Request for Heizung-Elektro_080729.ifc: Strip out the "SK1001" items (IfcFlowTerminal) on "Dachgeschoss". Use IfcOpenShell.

First a look at what the model holds.

```python
import ifcopenshell
import ifcopenshell.util.element

model = ifcopenshell.open("Heizung-Elektro_080729.ifc")
print(model.schema)
storey = next(s for s in model.by_type("IfcBuildingStorey") if s.Name == "Dachgeschoss")
terminals = [e for e in ifcopenshell.util.element.get_decomposition(storey) if e.is_a("IfcFlowTerminal")]
seen = {}
for e in terminals:
    element_type = ifcopenshell.util.element.get_type(e)
    name = element_type.Name if element_type not in (None, e) else None
    seen[name] = seen.get(name, 0) + 1
for name, count in sorted(seen.items(), key=str):
    print(count, "x", name)
```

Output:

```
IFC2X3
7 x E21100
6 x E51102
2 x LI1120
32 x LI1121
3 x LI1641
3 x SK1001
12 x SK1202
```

```python
import ifcopenshell
import ifcopenshell.api.root
import ifcopenshell.util.element

model = ifcopenshell.open("Heizung-Elektro_080729.ifc")

storey = next(s for s in model.by_type("IfcBuildingStorey") if s.Name == "Dachgeschoss")
terminals = [e for e in ifcopenshell.util.element.get_decomposition(storey) if e.is_a("IfcFlowTerminal")]
targets = [e for e in terminals if (t := ifcopenshell.util.element.get_type(e)) not in (None, e) and t.Name == "SK1001"]

for e in targets:
    ifcopenshell.api.root.remove_product(model, product=e)
print(len(targets), "removed")

model.write("Heizung-Elektro_080729_updated.ifc")
```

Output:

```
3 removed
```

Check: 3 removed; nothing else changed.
